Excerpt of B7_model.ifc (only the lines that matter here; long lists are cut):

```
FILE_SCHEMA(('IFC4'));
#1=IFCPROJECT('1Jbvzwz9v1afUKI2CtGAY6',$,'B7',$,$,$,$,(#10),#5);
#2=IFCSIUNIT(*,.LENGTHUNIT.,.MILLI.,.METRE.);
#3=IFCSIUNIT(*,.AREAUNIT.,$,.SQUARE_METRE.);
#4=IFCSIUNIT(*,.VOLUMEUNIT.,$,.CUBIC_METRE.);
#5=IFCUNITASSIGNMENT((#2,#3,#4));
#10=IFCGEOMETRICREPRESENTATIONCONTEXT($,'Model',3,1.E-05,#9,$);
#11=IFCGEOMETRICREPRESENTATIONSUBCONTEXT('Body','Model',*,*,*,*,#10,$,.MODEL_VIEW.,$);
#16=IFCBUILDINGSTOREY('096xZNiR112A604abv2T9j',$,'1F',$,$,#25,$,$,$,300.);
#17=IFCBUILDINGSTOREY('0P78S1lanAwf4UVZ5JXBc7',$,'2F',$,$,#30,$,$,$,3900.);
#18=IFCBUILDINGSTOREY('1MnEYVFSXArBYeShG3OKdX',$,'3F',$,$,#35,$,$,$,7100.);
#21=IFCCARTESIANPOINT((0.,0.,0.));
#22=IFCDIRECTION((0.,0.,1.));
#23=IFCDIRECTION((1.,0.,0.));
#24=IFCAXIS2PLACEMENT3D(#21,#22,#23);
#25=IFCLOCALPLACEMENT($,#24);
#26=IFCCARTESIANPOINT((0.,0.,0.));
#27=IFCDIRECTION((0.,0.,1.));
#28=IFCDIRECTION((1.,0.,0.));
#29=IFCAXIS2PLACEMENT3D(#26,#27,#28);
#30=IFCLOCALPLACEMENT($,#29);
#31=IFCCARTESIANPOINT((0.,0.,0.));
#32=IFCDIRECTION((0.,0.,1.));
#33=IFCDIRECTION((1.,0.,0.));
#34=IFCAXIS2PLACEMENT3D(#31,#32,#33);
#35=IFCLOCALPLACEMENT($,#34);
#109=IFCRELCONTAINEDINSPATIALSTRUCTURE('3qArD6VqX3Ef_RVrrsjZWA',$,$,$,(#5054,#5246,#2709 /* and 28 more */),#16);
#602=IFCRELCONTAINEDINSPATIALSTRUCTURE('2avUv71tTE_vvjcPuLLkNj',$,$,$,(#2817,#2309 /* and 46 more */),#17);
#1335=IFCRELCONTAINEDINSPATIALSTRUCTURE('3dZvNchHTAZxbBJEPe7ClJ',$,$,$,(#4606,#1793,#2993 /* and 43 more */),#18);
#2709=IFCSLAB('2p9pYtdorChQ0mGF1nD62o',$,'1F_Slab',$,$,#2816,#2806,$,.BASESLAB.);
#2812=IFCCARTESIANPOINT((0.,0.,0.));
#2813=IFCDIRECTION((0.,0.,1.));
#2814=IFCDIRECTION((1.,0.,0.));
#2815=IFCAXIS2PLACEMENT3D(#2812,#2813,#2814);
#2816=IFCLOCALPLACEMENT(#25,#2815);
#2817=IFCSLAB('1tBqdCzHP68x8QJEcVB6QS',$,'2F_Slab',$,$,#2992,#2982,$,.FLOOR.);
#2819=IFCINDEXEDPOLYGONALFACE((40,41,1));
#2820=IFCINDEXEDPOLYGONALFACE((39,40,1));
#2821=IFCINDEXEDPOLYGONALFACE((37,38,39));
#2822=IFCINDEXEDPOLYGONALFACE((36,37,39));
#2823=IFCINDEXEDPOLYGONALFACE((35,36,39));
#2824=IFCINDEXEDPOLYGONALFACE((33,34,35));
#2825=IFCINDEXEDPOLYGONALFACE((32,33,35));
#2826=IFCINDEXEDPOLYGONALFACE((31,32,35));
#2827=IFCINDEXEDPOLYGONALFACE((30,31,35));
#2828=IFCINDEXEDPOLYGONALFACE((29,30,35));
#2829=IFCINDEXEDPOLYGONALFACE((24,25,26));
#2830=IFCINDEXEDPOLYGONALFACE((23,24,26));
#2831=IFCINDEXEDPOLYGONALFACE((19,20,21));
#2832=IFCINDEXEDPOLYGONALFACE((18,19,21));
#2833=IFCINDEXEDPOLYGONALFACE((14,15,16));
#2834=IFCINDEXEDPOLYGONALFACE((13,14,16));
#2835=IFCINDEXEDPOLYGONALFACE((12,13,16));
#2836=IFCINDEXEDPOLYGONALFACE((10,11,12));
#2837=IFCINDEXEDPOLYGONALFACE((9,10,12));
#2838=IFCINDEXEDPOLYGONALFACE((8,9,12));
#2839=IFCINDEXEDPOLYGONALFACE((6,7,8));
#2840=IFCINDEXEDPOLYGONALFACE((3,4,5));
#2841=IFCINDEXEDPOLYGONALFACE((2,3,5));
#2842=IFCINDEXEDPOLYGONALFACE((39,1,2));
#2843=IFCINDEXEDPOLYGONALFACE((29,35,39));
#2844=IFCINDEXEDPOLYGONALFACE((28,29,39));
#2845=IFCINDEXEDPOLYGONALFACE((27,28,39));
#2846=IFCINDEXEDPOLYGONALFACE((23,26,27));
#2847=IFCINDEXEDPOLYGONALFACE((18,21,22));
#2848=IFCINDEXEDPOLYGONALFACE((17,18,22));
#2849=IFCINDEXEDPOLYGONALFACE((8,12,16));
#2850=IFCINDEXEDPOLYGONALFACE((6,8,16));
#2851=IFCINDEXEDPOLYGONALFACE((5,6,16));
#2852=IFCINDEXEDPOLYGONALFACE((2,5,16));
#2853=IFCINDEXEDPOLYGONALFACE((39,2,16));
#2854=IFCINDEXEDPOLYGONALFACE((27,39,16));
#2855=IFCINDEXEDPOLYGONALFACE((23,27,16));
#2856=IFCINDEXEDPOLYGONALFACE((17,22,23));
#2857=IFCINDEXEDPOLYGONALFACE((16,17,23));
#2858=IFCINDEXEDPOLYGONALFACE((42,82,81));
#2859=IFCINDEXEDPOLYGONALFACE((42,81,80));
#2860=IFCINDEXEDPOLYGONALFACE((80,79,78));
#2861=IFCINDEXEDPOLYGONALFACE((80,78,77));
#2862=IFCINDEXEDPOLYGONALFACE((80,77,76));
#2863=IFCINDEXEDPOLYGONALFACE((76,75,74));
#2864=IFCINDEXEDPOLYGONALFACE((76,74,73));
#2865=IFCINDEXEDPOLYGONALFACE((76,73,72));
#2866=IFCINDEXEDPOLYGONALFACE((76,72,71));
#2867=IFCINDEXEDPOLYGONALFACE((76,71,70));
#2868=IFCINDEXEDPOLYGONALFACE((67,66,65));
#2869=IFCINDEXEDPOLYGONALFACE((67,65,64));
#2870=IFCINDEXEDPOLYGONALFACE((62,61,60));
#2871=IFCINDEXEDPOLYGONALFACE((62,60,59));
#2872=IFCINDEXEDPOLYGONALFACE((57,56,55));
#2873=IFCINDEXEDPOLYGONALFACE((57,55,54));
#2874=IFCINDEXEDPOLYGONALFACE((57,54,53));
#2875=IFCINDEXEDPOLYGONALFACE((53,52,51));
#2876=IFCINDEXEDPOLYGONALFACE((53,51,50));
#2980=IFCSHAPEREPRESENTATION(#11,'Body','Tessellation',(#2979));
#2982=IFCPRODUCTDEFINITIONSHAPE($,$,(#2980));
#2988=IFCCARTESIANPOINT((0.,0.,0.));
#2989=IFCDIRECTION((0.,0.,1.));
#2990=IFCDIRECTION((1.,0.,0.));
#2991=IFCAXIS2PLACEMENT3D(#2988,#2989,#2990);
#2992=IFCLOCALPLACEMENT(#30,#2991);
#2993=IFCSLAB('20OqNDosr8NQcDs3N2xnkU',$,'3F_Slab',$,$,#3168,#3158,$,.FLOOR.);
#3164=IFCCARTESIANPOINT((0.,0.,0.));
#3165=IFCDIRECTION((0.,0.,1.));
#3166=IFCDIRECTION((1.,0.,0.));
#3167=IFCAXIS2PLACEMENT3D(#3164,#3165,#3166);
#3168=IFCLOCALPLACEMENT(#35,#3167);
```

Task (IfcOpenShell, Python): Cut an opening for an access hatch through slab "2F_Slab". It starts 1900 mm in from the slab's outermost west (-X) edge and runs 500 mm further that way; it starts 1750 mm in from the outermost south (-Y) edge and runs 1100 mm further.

```python
import numpy as np
import ifcopenshell
import ifcopenshell.api.feature
import ifcopenshell.api.geometry
import ifcopenshell.api.root
import ifcopenshell.geom
import ifcopenshell.util.placement
import ifcopenshell.util.representation
import ifcopenshell.util.shape
import ifcopenshell.util.unit

model = ifcopenshell.open("B7_model.ifc")
unit_scale = ifcopenshell.util.unit.calculate_unit_scale(model)
settings = ifcopenshell.geom.settings()


def volume(element):
    """Net volume in cubic metres, openings subtracted."""
    shape = ifcopenshell.geom.create_shape(settings, element)
    return ifcopenshell.util.shape.get_volume(shape.geometry)


slab = model.by_guid("1tBqdCzHP68x8QJEcVB6QS")
before = volume(slab)

# Extent in the slab's own axes, in metres. The edges named are its -X and -Y sides.
slab_shape = ifcopenshell.geom.create_shape(settings, slab)
vertices = ifcopenshell.util.shape.get_vertices(slab_shape.geometry)
x_min, y_min, bottom = vertices.min(axis=0)
top = vertices[:, 2].max()

opening = ifcopenshell.api.root.create_entity(model, ifc_class="IfcOpeningElement", name="Access hatch opening", predefined_type="OPENING")
context = ifcopenshell.util.representation.get_context(model, "Model", "Body", "MODEL_VIEW")
width, depth = 0.5, 1.1
outline = [(0.0, 0.0), (width, 0.0), (width, depth), (0.0, depth), (0.0, 0.0)]
# Overshoot both faces by 50 mm so the cut is clean.
shape = ifcopenshell.api.geometry.add_slab_representation(
    model, context=context, depth=top - bottom + 0.1, polyline=outline
)
ifcopenshell.api.geometry.assign_representation(model, product=opening, representation=shape)

matrix = ifcopenshell.util.placement.get_local_placement(slab.ObjectPlacement)
matrix[:, 3] = matrix @ np.append(np.array([x_min + 1.9, y_min + 1.75, bottom - 0.05]) / unit_scale, 1.0)
ifcopenshell.api.geometry.edit_object_placement(model, product=opening, matrix=matrix, is_si=False)
ifcopenshell.api.feature.add_feature(model, feature=opening, element=slab)

after = volume(slab)

print(f"slab volume {before:.3f} -> {after:.3f} m3")

model.write("B7_model-out.ifc")
```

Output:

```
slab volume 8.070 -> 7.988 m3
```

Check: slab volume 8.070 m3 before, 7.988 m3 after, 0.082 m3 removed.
